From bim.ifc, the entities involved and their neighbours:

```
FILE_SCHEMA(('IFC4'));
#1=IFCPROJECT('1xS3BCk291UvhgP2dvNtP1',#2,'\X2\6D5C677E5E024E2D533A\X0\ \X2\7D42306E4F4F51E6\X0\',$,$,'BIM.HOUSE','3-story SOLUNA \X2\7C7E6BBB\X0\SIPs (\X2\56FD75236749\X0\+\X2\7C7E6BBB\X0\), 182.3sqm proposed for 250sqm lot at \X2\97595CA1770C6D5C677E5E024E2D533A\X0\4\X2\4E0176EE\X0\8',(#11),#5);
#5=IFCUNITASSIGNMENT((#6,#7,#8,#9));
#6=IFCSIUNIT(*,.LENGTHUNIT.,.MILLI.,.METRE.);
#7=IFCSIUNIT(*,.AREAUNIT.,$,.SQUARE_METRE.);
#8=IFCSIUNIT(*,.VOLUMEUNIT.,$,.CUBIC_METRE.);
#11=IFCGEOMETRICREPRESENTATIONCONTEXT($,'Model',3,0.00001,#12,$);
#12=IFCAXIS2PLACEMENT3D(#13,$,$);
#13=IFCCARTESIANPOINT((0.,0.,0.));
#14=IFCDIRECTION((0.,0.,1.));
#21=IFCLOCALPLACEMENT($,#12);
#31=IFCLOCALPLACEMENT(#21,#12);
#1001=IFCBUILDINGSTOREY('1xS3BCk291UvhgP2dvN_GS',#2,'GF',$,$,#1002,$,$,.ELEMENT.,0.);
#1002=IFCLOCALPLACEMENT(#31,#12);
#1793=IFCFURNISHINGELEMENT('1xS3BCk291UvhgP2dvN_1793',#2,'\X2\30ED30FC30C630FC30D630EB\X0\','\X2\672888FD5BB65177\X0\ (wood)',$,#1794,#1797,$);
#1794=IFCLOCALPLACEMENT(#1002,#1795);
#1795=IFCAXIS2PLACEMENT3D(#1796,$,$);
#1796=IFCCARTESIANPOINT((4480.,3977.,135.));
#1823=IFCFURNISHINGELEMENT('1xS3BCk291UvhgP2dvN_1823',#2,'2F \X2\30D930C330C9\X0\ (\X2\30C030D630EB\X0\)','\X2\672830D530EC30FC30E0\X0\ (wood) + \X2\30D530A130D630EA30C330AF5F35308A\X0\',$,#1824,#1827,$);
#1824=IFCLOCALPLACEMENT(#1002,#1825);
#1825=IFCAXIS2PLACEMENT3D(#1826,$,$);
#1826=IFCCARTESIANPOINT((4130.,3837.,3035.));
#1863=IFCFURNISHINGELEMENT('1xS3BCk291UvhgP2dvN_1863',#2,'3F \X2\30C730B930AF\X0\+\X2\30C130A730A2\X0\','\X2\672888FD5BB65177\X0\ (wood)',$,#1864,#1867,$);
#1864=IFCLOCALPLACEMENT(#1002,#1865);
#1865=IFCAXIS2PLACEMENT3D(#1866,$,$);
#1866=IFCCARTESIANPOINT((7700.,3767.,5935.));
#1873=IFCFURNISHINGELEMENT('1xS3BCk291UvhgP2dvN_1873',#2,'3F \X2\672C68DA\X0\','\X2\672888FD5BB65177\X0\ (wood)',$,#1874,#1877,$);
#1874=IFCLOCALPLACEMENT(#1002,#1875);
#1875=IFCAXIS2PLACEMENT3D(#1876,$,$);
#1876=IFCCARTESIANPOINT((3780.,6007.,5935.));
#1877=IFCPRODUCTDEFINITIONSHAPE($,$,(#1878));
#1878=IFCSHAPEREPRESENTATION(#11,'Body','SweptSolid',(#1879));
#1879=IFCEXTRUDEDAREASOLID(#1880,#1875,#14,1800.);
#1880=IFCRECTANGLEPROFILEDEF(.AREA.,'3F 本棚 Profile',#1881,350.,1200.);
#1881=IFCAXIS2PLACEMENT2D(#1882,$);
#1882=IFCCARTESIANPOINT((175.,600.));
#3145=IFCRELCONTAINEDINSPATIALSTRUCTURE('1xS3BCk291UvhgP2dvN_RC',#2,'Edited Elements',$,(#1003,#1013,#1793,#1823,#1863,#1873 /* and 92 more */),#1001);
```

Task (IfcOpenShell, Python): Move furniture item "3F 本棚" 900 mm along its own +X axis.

```python
import ifcopenshell
import ifcopenshell.api.geometry
import ifcopenshell.util.placement

model = ifcopenshell.open("bim.ifc")

item = model.by_guid("1xS3BCk291UvhgP2dvN_1873")
matrix = ifcopenshell.util.placement.get_local_placement(item.ObjectPlacement)
matrix[:3, 3] += matrix[:3, 0] * 900.0
ifcopenshell.api.geometry.edit_object_placement(model, product=item, matrix=matrix, is_si=False)

print(ifcopenshell.util.placement.get_local_placement(item.ObjectPlacement).round(3) + 0.0)

model.write("bim_edited.ifc")
```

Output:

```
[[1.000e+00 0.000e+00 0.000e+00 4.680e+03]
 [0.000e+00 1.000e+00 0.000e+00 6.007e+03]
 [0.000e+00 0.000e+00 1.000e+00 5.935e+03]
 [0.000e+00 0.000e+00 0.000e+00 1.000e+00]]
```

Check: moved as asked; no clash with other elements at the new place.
